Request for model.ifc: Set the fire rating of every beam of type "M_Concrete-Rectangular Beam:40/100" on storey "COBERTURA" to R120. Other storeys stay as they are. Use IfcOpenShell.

First a look at what the model holds.

```python
import ifcopenshell
import ifcopenshell.util.element

model = ifcopenshell.open("model.ifc")
print(model.schema)
storey = next(s for s in model.by_type("IfcBuildingStorey") if s.Name == "COBERTURA")
beams = [e for e in ifcopenshell.util.element.get_decomposition(storey) if e.is_a("IfcBeam")]
seen = {}
for e in beams:
    element_type = ifcopenshell.util.element.get_type(e)
    key = (element_type.Name if element_type != e and element_type else None, ifcopenshell.util.element.get_pset(e, "Pset_BeamCommon", "FireRating"))
    seen[key] = seen.get(key, 0) + 1
for (name, value), count in sorted(seen.items(), key=str):
    print(count, "x", name, "|", value)
```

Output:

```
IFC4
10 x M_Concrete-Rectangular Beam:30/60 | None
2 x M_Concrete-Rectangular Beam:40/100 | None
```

```python
import ifcopenshell
import ifcopenshell.api.pset
import ifcopenshell.util.element

model = ifcopenshell.open("model.ifc")

storey = next(s for s in model.by_type("IfcBuildingStorey") if s.Name == "COBERTURA")
beams = [e for e in ifcopenshell.util.element.get_decomposition(storey) if e.is_a("IfcBeam")]

count = 0
for e in beams:
    element_type = ifcopenshell.util.element.get_type(e)
    if element_type in (None, e) or element_type.Name != "M_Concrete-Rectangular Beam:40/100":
        continue
    # add_pset returns the element's existing set when there is one.
    pset = ifcopenshell.api.pset.add_pset(model, product=e, name="Pset_BeamCommon")
    ifcopenshell.api.pset.edit_pset(model, pset=pset, properties={"FireRating": "R120"})
    count += 1

print(count, "beams updated")

model.write("model-out.ifc")
```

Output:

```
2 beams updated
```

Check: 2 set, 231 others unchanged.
